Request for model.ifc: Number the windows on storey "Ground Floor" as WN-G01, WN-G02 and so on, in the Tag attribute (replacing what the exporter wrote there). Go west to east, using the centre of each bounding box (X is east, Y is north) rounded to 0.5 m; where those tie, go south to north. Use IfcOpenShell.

First a look at what the model holds.

```python
import ifcopenshell
import ifcopenshell.util.element
import ifcopenshell.util.placement

model = ifcopenshell.open("model.ifc")
print(model.schema)
storey = next(s for s in model.by_type("IfcBuildingStorey") if s.Name == "Ground Floor")
windows = [e for e in ifcopenshell.util.element.get_decomposition(storey) if e.is_a("IfcWindow")]
for e in sorted(windows, key=lambda e: e.id()):
    origin = ifcopenshell.util.placement.get_local_placement(e.ObjectPlacement)[:3, 3]
    print(e.id(), e.Tag, e.Name, origin.round(2) + 0.0, sep=" | ")
```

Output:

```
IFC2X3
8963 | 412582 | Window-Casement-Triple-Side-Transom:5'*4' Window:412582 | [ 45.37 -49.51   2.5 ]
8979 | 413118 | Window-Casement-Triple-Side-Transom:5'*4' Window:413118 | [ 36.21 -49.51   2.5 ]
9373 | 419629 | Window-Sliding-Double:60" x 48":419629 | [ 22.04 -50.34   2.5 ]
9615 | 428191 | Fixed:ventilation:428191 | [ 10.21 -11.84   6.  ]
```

```python
import ifcopenshell
import ifcopenshell.geom
import ifcopenshell.util.element
import ifcopenshell.util.shape

model = ifcopenshell.open("model.ifc")
settings = ifcopenshell.geom.settings()
settings.set("use-world-coords", True)


def centre(element):
    shape = ifcopenshell.geom.create_shape(settings, element)
    return ifcopenshell.util.shape.get_bbox_centroid(shape.geometry)


storey = next(s for s in model.by_type("IfcBuildingStorey") if s.Name == "Ground Floor")
windows = [e for e in ifcopenshell.util.element.get_decomposition(storey) if e.is_a("IfcWindow")]

# Insertion points can sit at a corner or the storey origin, so sort by the geometry (in metres).
centres = {e: centre(e) for e in windows}
windows.sort(key=lambda e: (round(centres[e][0] / 0.5), centres[e][1]))

for i, e in enumerate(windows, start=1):
    number = f"WN-G{i:02d}"
    e.Tag = number
    print(e.id(), number)

model.write("model_updated.ifc")
```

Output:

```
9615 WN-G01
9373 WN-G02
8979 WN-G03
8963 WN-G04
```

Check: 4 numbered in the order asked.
